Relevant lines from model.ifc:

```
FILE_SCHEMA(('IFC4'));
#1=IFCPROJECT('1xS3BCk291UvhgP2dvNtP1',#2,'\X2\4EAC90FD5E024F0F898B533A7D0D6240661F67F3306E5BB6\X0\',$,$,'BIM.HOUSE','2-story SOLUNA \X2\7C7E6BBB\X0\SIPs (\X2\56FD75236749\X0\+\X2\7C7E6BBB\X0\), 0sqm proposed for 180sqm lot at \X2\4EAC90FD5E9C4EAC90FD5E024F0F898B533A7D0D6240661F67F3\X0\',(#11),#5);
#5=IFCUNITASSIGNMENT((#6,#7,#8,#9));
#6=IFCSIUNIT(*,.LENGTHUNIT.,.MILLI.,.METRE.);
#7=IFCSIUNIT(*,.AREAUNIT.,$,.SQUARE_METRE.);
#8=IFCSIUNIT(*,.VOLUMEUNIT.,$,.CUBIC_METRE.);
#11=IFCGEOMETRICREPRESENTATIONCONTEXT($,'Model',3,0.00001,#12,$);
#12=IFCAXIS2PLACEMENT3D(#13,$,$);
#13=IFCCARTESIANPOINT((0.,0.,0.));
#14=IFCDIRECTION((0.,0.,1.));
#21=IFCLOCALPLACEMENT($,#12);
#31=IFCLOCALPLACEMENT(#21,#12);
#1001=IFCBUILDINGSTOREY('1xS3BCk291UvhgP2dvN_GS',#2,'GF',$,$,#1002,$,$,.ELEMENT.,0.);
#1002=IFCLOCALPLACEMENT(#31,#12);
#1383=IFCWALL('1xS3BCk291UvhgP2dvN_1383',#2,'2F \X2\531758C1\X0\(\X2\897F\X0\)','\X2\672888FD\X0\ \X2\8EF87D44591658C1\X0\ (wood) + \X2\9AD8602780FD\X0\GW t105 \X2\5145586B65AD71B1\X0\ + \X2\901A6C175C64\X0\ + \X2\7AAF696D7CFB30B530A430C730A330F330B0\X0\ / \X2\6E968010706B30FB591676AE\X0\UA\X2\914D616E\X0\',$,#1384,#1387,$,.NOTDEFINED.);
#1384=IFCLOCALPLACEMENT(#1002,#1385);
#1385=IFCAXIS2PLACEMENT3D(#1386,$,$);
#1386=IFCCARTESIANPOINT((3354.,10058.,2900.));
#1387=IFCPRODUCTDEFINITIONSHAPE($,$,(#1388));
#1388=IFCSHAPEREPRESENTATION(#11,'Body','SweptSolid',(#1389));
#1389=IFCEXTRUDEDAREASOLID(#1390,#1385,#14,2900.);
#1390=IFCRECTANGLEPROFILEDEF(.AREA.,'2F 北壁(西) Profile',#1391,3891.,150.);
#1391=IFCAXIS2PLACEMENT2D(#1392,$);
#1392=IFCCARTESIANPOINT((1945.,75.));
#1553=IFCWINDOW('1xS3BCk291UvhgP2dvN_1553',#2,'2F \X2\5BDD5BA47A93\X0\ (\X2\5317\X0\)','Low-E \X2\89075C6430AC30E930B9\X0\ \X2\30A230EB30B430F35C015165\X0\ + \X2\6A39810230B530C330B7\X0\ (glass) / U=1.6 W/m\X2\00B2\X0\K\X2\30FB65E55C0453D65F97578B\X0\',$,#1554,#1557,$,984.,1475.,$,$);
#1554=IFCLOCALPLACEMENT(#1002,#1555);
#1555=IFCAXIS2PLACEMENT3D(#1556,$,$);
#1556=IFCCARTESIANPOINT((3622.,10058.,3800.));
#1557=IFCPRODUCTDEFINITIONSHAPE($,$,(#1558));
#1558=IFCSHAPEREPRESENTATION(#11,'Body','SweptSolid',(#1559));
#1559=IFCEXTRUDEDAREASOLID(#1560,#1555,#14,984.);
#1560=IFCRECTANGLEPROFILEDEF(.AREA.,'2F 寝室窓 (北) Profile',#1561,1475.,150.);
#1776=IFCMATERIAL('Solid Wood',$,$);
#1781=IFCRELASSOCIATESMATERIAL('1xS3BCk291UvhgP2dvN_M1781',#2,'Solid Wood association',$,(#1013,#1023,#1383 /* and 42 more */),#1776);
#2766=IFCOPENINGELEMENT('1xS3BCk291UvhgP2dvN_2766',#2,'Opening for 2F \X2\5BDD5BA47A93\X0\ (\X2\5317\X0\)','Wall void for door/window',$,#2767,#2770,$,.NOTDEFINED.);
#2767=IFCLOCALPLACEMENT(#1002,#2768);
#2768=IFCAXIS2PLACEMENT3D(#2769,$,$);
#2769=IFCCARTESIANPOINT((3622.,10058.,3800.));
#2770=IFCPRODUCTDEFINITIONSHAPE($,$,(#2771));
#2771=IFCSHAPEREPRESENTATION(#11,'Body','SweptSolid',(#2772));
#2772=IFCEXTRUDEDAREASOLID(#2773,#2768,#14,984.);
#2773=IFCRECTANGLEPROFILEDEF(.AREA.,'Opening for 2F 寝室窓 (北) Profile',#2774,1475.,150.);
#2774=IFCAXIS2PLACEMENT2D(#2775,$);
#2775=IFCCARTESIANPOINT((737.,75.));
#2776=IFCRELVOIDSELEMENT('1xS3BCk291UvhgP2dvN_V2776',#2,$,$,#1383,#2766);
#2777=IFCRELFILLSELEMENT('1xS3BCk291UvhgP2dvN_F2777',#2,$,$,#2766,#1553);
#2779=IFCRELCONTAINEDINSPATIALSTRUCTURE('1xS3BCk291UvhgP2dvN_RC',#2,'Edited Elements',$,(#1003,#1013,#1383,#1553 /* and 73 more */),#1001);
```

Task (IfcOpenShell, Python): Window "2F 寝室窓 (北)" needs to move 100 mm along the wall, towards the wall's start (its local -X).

```python
import ifcopenshell
import ifcopenshell.api.geometry
import ifcopenshell.util.placement

model = ifcopenshell.open("model.ifc")

window = model.by_guid("1xS3BCk291UvhgP2dvN_1553")
opening = window.FillsVoids[0].RelatingOpeningElement
wall = opening.VoidsElements[0].RelatingBuildingElement

wall_matrix = ifcopenshell.util.placement.get_local_placement(wall.ObjectPlacement)
shift = wall_matrix[:3, 0] * -100.0
before = ifcopenshell.util.placement.get_local_placement(window.ObjectPlacement)[:3, 3].copy()

# The window is not placed relative to its opening, so move both.
for product in (opening, window):
    matrix = ifcopenshell.util.placement.get_local_placement(product.ObjectPlacement)
    matrix[:3, 3] += shift
    ifcopenshell.api.geometry.edit_object_placement(model, product=product, matrix=matrix, is_si=False)

after = ifcopenshell.util.placement.get_local_placement(window.ObjectPlacement)[:3, 3]
print("window moved by", (after - before).round(3) + 0.0)

model.write("model_edited.ifc")
```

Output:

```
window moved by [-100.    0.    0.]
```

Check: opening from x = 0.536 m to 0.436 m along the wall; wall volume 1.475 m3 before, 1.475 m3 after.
